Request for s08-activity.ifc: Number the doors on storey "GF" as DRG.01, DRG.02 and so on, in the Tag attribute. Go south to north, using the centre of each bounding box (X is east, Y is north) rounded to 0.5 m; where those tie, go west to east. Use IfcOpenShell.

First a look at what the model holds.

```python
import ifcopenshell
import ifcopenshell.util.element
import ifcopenshell.util.placement

model = ifcopenshell.open("s08-activity.ifc")
print(model.schema)
storey = next(s for s in model.by_type("IfcBuildingStorey") if s.Name == "GF")
doors = [e for e in ifcopenshell.util.element.get_decomposition(storey) if e.is_a("IfcDoor")]
for e in sorted(doors, key=lambda e: e.id()):
    origin = ifcopenshell.util.placement.get_local_placement(e.ObjectPlacement)[:3, 3]
    print(e.id(), e.Tag, e.Name, origin.round(2) + 0.0, sep=" | ")
```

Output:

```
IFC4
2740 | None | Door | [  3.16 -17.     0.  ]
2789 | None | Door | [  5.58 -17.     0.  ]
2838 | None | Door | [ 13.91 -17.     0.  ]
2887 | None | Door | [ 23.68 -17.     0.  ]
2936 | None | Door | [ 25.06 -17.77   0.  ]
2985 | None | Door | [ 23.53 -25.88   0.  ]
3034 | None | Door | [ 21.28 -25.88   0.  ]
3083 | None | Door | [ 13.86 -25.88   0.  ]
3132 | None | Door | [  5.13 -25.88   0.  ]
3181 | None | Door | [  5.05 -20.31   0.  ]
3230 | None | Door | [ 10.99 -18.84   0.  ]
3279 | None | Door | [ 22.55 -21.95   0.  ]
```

```python
import ifcopenshell
import ifcopenshell.geom
import ifcopenshell.util.element
import ifcopenshell.util.shape

model = ifcopenshell.open("s08-activity.ifc")
settings = ifcopenshell.geom.settings()
settings.set("use-world-coords", True)


def centre(element):
    shape = ifcopenshell.geom.create_shape(settings, element)
    return ifcopenshell.util.shape.get_bbox_centroid(shape.geometry)


storey = next(s for s in model.by_type("IfcBuildingStorey") if s.Name == "GF")
doors = [e for e in ifcopenshell.util.element.get_decomposition(storey) if e.is_a("IfcDoor")]

# Insertion points can sit at a corner or the storey origin, so sort by the geometry (in metres).
centres = {e: centre(e) for e in doors}
doors.sort(key=lambda e: (round(centres[e][1] / 0.5), centres[e][0]))

for i, e in enumerate(doors, start=1):
    number = f"DRG.{i:02d}"
    e.Tag = number
    print(e.id(), number)

model.write("s08-activity_updated.ifc")
```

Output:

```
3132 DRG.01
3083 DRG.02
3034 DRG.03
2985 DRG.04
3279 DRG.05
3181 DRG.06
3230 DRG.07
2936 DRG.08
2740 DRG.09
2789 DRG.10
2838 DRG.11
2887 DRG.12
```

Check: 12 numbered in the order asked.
